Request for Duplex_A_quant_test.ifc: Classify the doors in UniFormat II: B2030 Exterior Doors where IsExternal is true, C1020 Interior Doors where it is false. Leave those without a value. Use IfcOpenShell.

First a look at what the model holds.

```python
import ifcopenshell
import ifcopenshell.util.element

model = ifcopenshell.open("Duplex_A_quant_test.ifc")
print(model.schema)
print("classifications:", [c.Name for c in model.by_type("IfcClassification")])
values = [ifcopenshell.util.element.get_pset(e, "Pset_DoorCommon", "IsExternal") for e in model.by_type("IfcDoor")]
for value in (True, False, None):
    print("IsExternal", value, values.count(value))
```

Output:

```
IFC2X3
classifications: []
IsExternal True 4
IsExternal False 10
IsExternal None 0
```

```python
import ifcopenshell
import ifcopenshell.api.classification
import ifcopenshell.util.element

model = ifcopenshell.open("Duplex_A_quant_test.ifc")

# IFC2X3 requires Source and Edition and has no link from the project to the system.
system = model.create_entity("IfcClassification", Source="ASTM", Edition="E1557", Name="UniFormat II")

doors = model.by_type("IfcDoor")
external = {e: ifcopenshell.util.element.get_pset(e, "Pset_DoorCommon", "IsExternal") for e in doors}
for flag, code, name in ((True, "B2030", "Exterior Doors"), (False, "C1020", "Interior Doors")):
    products = [e for e in doors if external[e] is flag]
    ifcopenshell.api.classification.add_reference(
        model, products=products, classification=system, identification=code, name=name
    )
    print(code, len(products))

model.write("Duplex_A_quant_test_v2.ifc")
```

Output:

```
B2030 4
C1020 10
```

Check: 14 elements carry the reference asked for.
